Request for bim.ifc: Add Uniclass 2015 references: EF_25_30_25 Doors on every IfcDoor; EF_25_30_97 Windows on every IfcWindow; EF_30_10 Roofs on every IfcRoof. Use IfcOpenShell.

First a look at what the model holds.

```python
import ifcopenshell

model = ifcopenshell.open("bim.ifc")
print(model.schema)
print("classifications:", [c.Name for c in model.by_type("IfcClassification")])
for ifc_class in ("IfcDoor", "IfcRoof", "IfcStair", "IfcWall", "IfcWindow"):
    print(ifc_class, len(model.by_type(ifc_class)))
```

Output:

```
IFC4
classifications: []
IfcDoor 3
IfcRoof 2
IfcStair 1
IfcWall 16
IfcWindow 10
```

```python
import ifcopenshell
import ifcopenshell.api.classification

model = ifcopenshell.open("bim.ifc")

system = ifcopenshell.api.classification.add_classification(model, classification="Uniclass 2015")

codes = {
    "IfcDoor": ("EF_25_30_25", "Doors"),
    "IfcWindow": ("EF_25_30_97", "Windows"),
    "IfcRoof": ("EF_30_10", "Roofs"),
}
for ifc_class, (code, name) in codes.items():
    products = model.by_type(ifc_class)
    ifcopenshell.api.classification.add_reference(
        model, products=products, classification=system, identification=code, name=name
    )
    print(code, len(products))

model.write("bim_updated.ifc")
```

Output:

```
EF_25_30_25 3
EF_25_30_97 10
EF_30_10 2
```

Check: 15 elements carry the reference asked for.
